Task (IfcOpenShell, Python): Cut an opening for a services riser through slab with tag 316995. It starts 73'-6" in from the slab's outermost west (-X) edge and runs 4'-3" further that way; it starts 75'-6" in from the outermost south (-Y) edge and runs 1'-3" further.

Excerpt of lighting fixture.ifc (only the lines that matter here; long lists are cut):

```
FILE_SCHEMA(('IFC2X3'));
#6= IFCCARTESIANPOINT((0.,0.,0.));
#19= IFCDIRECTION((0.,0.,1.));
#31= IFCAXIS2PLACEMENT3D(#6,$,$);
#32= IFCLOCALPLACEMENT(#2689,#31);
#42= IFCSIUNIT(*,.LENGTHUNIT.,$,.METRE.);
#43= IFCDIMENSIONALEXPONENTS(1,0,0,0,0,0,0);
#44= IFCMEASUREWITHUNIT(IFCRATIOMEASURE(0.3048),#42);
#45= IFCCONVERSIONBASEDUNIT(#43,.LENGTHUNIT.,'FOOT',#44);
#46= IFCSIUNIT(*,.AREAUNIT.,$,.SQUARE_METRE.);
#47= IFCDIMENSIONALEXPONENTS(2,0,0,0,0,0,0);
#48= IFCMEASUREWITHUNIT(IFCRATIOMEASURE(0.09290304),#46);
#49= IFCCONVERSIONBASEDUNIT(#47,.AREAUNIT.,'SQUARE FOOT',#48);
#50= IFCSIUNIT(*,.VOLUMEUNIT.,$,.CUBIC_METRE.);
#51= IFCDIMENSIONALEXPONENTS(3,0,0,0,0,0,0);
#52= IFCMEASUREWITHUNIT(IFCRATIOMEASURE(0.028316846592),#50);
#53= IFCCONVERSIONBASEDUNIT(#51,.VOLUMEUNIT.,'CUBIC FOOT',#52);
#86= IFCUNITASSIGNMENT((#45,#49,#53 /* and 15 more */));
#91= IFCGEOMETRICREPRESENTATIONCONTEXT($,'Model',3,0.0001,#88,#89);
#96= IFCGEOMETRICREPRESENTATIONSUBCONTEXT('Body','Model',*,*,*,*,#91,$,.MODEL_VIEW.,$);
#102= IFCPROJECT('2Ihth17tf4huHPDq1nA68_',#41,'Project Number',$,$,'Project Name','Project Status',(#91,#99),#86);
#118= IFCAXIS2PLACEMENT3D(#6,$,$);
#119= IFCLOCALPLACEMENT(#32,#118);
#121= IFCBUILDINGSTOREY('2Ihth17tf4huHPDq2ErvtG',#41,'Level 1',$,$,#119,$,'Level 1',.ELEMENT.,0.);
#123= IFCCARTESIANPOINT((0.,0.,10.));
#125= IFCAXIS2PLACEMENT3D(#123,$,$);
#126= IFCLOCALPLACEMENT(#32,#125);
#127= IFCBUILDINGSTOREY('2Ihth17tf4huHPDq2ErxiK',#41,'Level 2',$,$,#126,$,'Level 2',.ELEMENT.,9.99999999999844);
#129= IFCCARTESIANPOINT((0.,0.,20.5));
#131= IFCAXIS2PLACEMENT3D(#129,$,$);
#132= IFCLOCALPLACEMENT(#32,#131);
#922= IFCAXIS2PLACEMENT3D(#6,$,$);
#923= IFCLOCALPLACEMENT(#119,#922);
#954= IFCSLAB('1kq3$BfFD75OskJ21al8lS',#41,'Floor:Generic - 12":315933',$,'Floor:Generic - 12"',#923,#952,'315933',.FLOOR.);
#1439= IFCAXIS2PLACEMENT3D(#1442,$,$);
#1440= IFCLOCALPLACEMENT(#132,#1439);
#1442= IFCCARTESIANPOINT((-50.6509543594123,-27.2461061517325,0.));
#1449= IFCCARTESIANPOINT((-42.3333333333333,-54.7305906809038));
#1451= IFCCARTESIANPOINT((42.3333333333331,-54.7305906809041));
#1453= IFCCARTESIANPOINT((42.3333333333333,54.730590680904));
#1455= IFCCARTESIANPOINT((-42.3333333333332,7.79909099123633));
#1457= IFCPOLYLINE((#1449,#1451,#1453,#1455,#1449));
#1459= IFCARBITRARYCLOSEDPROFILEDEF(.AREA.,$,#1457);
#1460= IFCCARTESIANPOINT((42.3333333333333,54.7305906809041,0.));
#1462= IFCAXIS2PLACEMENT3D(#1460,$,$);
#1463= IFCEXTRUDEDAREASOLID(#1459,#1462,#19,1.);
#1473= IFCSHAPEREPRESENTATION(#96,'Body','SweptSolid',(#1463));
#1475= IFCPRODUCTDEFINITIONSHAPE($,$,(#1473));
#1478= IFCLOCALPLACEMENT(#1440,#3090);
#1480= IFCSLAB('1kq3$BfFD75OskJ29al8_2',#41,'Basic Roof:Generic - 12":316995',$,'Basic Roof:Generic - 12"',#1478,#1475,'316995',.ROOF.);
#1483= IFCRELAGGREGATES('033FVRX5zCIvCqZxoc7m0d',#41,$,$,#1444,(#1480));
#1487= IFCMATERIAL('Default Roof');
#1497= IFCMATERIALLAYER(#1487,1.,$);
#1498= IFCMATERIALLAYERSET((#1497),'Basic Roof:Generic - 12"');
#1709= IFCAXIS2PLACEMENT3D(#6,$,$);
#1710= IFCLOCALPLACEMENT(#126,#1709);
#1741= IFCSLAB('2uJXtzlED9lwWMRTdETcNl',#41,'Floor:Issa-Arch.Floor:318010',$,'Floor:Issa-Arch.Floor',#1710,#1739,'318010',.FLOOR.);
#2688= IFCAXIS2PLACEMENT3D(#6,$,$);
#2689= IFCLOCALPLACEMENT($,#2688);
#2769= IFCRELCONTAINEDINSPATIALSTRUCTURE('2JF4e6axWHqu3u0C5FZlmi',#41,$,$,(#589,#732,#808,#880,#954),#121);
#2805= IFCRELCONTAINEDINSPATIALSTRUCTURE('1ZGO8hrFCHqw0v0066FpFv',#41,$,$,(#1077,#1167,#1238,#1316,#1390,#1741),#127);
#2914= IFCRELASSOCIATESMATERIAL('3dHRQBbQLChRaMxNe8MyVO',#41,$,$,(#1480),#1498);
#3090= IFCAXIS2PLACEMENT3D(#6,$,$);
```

```python
import numpy as np
import ifcopenshell
import ifcopenshell.api.feature
import ifcopenshell.api.geometry
import ifcopenshell.api.root
import ifcopenshell.geom
import ifcopenshell.util.placement
import ifcopenshell.util.representation
import ifcopenshell.util.shape
import ifcopenshell.util.unit

model = ifcopenshell.open("lighting fixture.ifc")
unit_scale = ifcopenshell.util.unit.calculate_unit_scale(model)
settings = ifcopenshell.geom.settings()


def volume(element):
    """Net volume in cubic metres, openings subtracted."""
    shape = ifcopenshell.geom.create_shape(settings, element)
    return ifcopenshell.util.shape.get_volume(shape.geometry)


slab = model.by_id(1480)
before = volume(slab)

# Extent in the slab's own axes, in metres. The edges named are its -X and -Y sides.
slab_shape = ifcopenshell.geom.create_shape(settings, slab)
vertices = ifcopenshell.util.shape.get_vertices(slab_shape.geometry)
x_min, y_min, bottom = vertices.min(axis=0)
top = vertices[:, 2].max()

opening = ifcopenshell.api.root.create_entity(model, ifc_class="IfcOpeningElement", name="Services riser opening")
context = ifcopenshell.util.representation.get_context(model, "Model", "Body", "MODEL_VIEW")
width, depth = 1.2954, 0.381
outline = [(0.0, 0.0), (width, 0.0), (width, depth), (0.0, depth), (0.0, 0.0)]
# Overshoot both faces by 50 mm so the cut is clean.
shape = ifcopenshell.api.geometry.add_slab_representation(
    model, context=context, depth=top - bottom + 0.1, polyline=outline
)
ifcopenshell.api.geometry.assign_representation(model, product=opening, representation=shape)

matrix = ifcopenshell.util.placement.get_local_placement(slab.ObjectPlacement)
matrix[:, 3] = matrix @ np.append(np.array([x_min + 22.4028, y_min + 23.0124, bottom - 0.05]) / unit_scale, 1.0)
ifcopenshell.api.geometry.edit_object_placement(model, product=opening, matrix=matrix, is_si=False)
ifcopenshell.api.feature.add_feature(model, feature=opening, element=slab)

after = volume(slab)

print(f"slab volume {before:.3f} -> {after:.3f} m3")

model.write("lighting fixture_v2.ifc")
```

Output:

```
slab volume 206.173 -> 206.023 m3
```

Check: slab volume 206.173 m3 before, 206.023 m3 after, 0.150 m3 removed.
